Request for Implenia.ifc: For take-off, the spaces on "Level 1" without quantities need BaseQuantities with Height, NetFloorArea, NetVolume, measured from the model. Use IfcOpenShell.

First a look at what the model holds.

```python
import ifcopenshell
import ifcopenshell.util.element
import ifcopenshell.util.unit

model = ifcopenshell.open("Implenia.ifc")
print(model.schema)
for unit_type in ("LENGTHUNIT", "AREAUNIT", "VOLUMEUNIT"):
    print(unit_type, ifcopenshell.util.unit.calculate_unit_scale(model, unit_type))
storey = next(s for s in model.by_type("IfcBuildingStorey") if s.Name == "Level 1")
spaces = [e for e in ifcopenshell.util.element.get_decomposition(storey) if e.is_a("IfcSpace")]
for e in sorted(spaces, key=lambda e: e.id()):
    print(e.id(), e.is_a(), e.Name, list(ifcopenshell.util.element.get_psets(e, qtos_only=True)), sep=" | ")
```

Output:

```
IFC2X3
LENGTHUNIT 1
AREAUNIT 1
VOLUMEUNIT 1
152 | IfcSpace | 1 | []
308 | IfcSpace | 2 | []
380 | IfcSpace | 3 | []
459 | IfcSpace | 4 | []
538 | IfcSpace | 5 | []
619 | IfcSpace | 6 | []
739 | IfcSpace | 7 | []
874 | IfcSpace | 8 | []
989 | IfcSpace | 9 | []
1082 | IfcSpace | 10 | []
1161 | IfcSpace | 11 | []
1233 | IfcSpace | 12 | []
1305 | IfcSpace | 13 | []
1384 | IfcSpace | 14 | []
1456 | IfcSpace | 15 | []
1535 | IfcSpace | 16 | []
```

```python
import ifcopenshell
import ifcopenshell.api.pset
import ifcopenshell.geom
import ifcopenshell.util.element
import ifcopenshell.util.shape
import ifcopenshell.util.unit

model = ifcopenshell.open("Implenia.ifc")
unit_scale = ifcopenshell.util.unit.calculate_unit_scale(model)
area_scale = ifcopenshell.util.unit.calculate_unit_scale(model, "AREAUNIT")
volume_scale = ifcopenshell.util.unit.calculate_unit_scale(model, "VOLUMEUNIT")
settings = ifcopenshell.geom.settings()

storey = next(s for s in model.by_type("IfcBuildingStorey") if s.Name == "Level 1")
spaces = [e for e in ifcopenshell.util.element.get_decomposition(storey) if e.is_a("IfcSpace")]

for e in sorted(spaces, key=lambda e: e.id()):
    if ifcopenshell.util.element.get_psets(e, qtos_only=True, should_inherit=False):
        continue
    # Geometry comes back in metres, in the element's own axes.
    shape = ifcopenshell.geom.create_shape(settings, e)
    values = {
        "Height": ifcopenshell.util.shape.get_z(shape.geometry) / unit_scale,
        "NetFloorArea": ifcopenshell.util.shape.get_footprint_area(shape.geometry) / area_scale,
        "NetVolume": ifcopenshell.util.shape.get_volume(shape.geometry) / volume_scale,
    }
    qto = ifcopenshell.api.pset.add_qto(model, product=e, name="BaseQuantities")
    ifcopenshell.api.pset.edit_qto(model, qto=qto, properties=values)
    print(e.id(), {k: round(v, 3) for k, v in values.items()})

model.write("Implenia_v2.ifc")
```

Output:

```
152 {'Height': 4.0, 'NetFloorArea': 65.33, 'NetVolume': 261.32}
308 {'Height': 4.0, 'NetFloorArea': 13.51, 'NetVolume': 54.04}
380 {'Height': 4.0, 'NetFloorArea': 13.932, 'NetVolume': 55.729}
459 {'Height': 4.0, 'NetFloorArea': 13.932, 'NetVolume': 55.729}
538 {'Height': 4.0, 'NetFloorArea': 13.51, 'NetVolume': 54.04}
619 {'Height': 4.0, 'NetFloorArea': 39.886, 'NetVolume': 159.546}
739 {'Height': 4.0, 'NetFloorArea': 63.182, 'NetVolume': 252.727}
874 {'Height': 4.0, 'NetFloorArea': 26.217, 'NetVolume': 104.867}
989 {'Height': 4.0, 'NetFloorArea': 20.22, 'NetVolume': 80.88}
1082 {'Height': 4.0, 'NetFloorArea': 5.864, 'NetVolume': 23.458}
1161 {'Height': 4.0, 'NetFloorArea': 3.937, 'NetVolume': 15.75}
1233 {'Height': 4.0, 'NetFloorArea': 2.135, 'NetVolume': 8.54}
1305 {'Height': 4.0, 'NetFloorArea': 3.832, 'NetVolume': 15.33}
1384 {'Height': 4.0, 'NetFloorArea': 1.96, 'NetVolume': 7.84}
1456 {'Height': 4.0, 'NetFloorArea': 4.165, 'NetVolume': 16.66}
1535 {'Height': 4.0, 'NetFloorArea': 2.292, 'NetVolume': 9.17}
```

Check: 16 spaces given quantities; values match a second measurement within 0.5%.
